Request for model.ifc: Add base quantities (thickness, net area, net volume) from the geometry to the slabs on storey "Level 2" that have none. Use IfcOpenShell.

First a look at what the model holds.

```python
import ifcopenshell
import ifcopenshell.util.element
import ifcopenshell.util.unit

model = ifcopenshell.open("model.ifc")
print(model.schema)
for unit_type in ("LENGTHUNIT", "AREAUNIT", "VOLUMEUNIT"):
    print(unit_type, ifcopenshell.util.unit.calculate_unit_scale(model, unit_type))
storey = next(s for s in model.by_type("IfcBuildingStorey") if s.Name == "Level 2")
slabs = [e for e in ifcopenshell.util.element.get_decomposition(storey) if e.is_a("IfcSlab")]
for e in sorted(slabs, key=lambda e: e.id()):
    print(e.id(), e.is_a(), e.Name, list(ifcopenshell.util.element.get_psets(e, qtos_only=True)), sep=" | ")
```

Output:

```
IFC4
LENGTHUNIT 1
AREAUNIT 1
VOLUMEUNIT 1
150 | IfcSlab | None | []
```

```python
import ifcopenshell
import ifcopenshell.api.pset
import ifcopenshell.geom
import ifcopenshell.util.element
import ifcopenshell.util.shape
import ifcopenshell.util.unit

model = ifcopenshell.open("model.ifc")
unit_scale = ifcopenshell.util.unit.calculate_unit_scale(model)
area_scale = ifcopenshell.util.unit.calculate_unit_scale(model, "AREAUNIT")
volume_scale = ifcopenshell.util.unit.calculate_unit_scale(model, "VOLUMEUNIT")
settings = ifcopenshell.geom.settings()

storey = next(s for s in model.by_type("IfcBuildingStorey") if s.Name == "Level 2")
slabs = [e for e in ifcopenshell.util.element.get_decomposition(storey) if e.is_a("IfcSlab")]

for e in sorted(slabs, key=lambda e: e.id()):
    if ifcopenshell.util.element.get_psets(e, qtos_only=True, should_inherit=False):
        continue
    # Geometry comes back in metres, in the element's own axes.
    shape = ifcopenshell.geom.create_shape(settings, e)
    values = {
        "Width": ifcopenshell.util.shape.get_z(shape.geometry) / unit_scale,
        "NetArea": ifcopenshell.util.shape.get_footprint_area(shape.geometry) / area_scale,
        "NetVolume": ifcopenshell.util.shape.get_volume(shape.geometry) / volume_scale,
    }
    qto = ifcopenshell.api.pset.add_qto(model, product=e, name="Qto_SlabBaseQuantities")
    ifcopenshell.api.pset.edit_qto(model, qto=qto, properties=values)
    print(e.id(), {k: round(v, 3) for k, v in values.items()})

model.write("model_rev.ifc")
```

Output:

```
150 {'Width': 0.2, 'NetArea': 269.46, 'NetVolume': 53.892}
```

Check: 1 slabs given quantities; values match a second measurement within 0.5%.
